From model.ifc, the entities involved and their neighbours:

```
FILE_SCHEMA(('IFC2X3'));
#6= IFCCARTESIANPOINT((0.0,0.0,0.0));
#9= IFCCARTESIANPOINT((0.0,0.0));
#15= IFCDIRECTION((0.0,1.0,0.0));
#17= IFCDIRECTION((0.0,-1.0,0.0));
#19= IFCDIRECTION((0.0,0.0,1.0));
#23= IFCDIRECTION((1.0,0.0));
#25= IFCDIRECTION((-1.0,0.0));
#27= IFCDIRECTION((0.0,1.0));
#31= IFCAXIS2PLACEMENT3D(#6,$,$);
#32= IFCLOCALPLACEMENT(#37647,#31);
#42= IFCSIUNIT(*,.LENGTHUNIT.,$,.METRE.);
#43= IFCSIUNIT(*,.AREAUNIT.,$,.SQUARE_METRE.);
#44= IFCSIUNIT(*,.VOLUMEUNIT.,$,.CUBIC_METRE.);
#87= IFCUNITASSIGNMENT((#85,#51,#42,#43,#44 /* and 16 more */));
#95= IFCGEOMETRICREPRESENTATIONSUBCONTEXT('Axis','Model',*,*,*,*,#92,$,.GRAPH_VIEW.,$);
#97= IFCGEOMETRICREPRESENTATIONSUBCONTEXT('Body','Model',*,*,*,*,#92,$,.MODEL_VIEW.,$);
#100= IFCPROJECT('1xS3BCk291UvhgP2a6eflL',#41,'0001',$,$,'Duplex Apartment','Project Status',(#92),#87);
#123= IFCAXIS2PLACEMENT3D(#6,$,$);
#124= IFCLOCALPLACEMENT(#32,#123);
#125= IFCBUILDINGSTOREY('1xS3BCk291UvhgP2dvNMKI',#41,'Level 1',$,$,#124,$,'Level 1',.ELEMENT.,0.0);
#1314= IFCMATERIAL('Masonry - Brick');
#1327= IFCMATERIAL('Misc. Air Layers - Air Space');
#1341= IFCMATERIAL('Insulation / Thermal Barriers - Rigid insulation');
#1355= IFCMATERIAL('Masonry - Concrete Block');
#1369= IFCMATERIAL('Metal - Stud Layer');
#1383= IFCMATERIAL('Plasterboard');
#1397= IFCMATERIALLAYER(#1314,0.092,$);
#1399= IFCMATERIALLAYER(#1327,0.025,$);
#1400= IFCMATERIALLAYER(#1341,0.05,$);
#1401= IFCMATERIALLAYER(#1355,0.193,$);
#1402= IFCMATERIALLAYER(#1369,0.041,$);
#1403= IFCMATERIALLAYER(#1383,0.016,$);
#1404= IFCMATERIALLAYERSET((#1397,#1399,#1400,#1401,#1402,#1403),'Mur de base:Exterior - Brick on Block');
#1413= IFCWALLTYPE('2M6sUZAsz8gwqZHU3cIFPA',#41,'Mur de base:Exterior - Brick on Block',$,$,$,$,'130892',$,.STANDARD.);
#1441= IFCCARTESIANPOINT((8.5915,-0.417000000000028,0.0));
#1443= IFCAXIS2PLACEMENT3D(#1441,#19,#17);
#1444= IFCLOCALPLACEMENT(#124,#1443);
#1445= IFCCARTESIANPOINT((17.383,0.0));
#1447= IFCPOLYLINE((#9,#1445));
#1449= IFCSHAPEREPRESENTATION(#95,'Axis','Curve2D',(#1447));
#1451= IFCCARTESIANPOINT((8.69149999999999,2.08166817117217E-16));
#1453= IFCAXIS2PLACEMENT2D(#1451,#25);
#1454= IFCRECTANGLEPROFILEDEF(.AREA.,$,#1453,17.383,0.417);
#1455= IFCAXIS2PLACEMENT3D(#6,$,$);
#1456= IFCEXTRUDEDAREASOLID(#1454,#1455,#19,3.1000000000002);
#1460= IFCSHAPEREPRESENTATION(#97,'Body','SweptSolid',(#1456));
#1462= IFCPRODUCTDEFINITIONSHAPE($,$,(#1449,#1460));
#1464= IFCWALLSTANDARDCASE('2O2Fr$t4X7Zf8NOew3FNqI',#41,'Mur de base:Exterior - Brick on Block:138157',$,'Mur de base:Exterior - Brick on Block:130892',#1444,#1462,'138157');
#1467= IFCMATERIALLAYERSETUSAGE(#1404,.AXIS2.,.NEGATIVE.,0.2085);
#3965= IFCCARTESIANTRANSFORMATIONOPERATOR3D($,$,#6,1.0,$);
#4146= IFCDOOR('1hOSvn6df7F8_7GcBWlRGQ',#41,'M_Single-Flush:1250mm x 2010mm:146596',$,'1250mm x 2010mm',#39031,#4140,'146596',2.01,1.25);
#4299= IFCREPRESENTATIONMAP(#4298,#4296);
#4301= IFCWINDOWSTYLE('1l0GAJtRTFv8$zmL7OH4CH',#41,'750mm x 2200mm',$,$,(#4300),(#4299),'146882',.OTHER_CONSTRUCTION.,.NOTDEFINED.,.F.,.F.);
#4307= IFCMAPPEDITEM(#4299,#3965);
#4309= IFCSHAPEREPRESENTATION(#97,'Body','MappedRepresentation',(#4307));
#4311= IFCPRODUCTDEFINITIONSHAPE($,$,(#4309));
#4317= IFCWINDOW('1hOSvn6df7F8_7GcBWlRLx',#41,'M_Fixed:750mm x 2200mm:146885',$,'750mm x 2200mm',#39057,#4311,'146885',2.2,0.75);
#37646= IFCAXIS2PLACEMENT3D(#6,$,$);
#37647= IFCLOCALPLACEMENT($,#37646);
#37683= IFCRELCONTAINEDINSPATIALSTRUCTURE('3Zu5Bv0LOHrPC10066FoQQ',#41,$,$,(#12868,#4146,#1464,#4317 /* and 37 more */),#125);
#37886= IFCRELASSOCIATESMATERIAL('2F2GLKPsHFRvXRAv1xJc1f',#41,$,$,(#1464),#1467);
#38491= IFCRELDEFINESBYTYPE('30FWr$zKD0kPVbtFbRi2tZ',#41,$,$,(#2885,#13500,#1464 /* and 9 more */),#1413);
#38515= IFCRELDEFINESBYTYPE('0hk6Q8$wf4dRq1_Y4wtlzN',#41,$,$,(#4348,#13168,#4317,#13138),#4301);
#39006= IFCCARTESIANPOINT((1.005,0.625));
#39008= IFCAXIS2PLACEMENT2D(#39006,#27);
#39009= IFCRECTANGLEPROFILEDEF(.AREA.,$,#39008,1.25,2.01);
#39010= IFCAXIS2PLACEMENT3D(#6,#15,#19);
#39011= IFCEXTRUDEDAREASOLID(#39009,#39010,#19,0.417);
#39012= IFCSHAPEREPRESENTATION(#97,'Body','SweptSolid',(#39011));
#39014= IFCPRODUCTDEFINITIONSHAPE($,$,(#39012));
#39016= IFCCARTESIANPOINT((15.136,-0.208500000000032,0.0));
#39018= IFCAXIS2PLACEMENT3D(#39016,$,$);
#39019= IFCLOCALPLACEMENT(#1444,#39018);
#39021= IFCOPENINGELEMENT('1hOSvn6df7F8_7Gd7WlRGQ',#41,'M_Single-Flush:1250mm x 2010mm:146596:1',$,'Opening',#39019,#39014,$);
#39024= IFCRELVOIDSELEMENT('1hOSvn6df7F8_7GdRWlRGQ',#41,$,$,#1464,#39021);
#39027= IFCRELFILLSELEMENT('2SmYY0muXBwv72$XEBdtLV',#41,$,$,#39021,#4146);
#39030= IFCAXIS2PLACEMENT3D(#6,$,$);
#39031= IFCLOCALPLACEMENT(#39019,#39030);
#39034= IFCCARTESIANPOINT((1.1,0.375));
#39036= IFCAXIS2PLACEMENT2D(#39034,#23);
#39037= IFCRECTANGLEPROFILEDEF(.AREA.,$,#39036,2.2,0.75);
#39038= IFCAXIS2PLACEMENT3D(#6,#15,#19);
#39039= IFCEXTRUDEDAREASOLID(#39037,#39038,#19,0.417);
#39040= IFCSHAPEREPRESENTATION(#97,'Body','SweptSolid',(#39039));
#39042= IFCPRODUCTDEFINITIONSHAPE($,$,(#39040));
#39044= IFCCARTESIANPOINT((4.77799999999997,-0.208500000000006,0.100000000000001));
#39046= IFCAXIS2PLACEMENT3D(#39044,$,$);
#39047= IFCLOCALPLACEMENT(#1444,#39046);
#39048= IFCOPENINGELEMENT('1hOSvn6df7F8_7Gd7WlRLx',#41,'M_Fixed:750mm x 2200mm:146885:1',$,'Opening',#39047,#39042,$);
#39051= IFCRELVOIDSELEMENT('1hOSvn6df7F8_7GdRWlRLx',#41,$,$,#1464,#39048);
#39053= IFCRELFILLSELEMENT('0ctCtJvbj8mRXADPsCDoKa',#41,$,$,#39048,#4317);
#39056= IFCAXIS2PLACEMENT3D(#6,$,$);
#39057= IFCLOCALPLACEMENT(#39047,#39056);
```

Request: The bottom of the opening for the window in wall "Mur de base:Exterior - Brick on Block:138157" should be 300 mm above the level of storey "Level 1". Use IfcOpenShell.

```python
import numpy as np
import ifcopenshell
import ifcopenshell.api.geometry
import ifcopenshell.geom
import ifcopenshell.util.element
import ifcopenshell.util.placement
import ifcopenshell.util.shape
import ifcopenshell.util.unit

model = ifcopenshell.open("model.ifc")
unit_scale = ifcopenshell.util.unit.calculate_unit_scale(model)

window = model.by_guid("1hOSvn6df7F8_7GcBWlRLx")
opening = window.FillsVoids[0].RelatingOpeningElement
storey = ifcopenshell.util.element.get_container(window, ifc_class="IfcBuildingStorey")
level = ifcopenshell.util.placement.get_local_placement(storey.ObjectPlacement)[2, 3]

# The opening's origin need not be at the sill, so measure its lowest point.
shape = ifcopenshell.geom.create_shape(ifcopenshell.geom.settings(), opening)
bottom = ifcopenshell.util.shape.get_shape_bottom_elevation(shape, shape.geometry) / unit_scale
dz = level + 0.3 / unit_scale - bottom

shift = np.array([0.0, 0.0, dz])
# The window is placed relative to its opening, so it follows when the opening moves.
matrix = ifcopenshell.util.placement.get_local_placement(opening.ObjectPlacement)
matrix[:3, 3] += shift
ifcopenshell.api.geometry.edit_object_placement(
    model, product=opening, matrix=matrix, is_si=False, should_transform_children=True
)

print(f"moved by {dz * unit_scale:+.3f} m")

model.write("model_v2.ifc")
```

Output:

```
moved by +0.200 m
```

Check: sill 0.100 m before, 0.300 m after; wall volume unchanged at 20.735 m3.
